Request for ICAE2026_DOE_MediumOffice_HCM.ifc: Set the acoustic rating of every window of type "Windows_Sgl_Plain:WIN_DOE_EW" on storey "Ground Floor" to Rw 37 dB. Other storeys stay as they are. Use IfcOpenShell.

First a look at what the model holds.

```python
import ifcopenshell
import ifcopenshell.util.element

model = ifcopenshell.open("ICAE2026_DOE_MediumOffice_HCM.ifc")
print(model.schema)
storey = next(s for s in model.by_type("IfcBuildingStorey") if s.Name == "Ground Floor")
windows = [e for e in ifcopenshell.util.element.get_decomposition(storey) if e.is_a("IfcWindow")]
seen = {}
for e in windows:
    element_type = ifcopenshell.util.element.get_type(e)
    key = (element_type.Name if element_type != e and element_type else None, ifcopenshell.util.element.get_pset(e, "Pset_WindowCommon", "AcousticRating"))
    seen[key] = seen.get(key, 0) + 1
for (name, value), count in sorted(seen.items(), key=str):
    print(count, "x", name, "|", value)
```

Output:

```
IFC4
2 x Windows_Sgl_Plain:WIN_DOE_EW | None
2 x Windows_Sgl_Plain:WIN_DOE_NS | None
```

```python
import ifcopenshell
import ifcopenshell.api.pset
import ifcopenshell.util.element

model = ifcopenshell.open("ICAE2026_DOE_MediumOffice_HCM.ifc")

storey = next(s for s in model.by_type("IfcBuildingStorey") if s.Name == "Ground Floor")
windows = [e for e in ifcopenshell.util.element.get_decomposition(storey) if e.is_a("IfcWindow")]

count = 0
for e in windows:
    element_type = ifcopenshell.util.element.get_type(e)
    if element_type in (None, e) or element_type.Name != "Windows_Sgl_Plain:WIN_DOE_EW":
        continue
    # add_pset returns the element's existing set when there is one.
    pset = ifcopenshell.api.pset.add_pset(model, product=e, name="Pset_WindowCommon")
    ifcopenshell.api.pset.edit_pset(model, pset=pset, properties={"AcousticRating": "Rw 37 dB"})
    count += 1

print(count, "windows updated")

model.write("ICAE2026_DOE_MediumOffice_HCM_rev.ifc")
```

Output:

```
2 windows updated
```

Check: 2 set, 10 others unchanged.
